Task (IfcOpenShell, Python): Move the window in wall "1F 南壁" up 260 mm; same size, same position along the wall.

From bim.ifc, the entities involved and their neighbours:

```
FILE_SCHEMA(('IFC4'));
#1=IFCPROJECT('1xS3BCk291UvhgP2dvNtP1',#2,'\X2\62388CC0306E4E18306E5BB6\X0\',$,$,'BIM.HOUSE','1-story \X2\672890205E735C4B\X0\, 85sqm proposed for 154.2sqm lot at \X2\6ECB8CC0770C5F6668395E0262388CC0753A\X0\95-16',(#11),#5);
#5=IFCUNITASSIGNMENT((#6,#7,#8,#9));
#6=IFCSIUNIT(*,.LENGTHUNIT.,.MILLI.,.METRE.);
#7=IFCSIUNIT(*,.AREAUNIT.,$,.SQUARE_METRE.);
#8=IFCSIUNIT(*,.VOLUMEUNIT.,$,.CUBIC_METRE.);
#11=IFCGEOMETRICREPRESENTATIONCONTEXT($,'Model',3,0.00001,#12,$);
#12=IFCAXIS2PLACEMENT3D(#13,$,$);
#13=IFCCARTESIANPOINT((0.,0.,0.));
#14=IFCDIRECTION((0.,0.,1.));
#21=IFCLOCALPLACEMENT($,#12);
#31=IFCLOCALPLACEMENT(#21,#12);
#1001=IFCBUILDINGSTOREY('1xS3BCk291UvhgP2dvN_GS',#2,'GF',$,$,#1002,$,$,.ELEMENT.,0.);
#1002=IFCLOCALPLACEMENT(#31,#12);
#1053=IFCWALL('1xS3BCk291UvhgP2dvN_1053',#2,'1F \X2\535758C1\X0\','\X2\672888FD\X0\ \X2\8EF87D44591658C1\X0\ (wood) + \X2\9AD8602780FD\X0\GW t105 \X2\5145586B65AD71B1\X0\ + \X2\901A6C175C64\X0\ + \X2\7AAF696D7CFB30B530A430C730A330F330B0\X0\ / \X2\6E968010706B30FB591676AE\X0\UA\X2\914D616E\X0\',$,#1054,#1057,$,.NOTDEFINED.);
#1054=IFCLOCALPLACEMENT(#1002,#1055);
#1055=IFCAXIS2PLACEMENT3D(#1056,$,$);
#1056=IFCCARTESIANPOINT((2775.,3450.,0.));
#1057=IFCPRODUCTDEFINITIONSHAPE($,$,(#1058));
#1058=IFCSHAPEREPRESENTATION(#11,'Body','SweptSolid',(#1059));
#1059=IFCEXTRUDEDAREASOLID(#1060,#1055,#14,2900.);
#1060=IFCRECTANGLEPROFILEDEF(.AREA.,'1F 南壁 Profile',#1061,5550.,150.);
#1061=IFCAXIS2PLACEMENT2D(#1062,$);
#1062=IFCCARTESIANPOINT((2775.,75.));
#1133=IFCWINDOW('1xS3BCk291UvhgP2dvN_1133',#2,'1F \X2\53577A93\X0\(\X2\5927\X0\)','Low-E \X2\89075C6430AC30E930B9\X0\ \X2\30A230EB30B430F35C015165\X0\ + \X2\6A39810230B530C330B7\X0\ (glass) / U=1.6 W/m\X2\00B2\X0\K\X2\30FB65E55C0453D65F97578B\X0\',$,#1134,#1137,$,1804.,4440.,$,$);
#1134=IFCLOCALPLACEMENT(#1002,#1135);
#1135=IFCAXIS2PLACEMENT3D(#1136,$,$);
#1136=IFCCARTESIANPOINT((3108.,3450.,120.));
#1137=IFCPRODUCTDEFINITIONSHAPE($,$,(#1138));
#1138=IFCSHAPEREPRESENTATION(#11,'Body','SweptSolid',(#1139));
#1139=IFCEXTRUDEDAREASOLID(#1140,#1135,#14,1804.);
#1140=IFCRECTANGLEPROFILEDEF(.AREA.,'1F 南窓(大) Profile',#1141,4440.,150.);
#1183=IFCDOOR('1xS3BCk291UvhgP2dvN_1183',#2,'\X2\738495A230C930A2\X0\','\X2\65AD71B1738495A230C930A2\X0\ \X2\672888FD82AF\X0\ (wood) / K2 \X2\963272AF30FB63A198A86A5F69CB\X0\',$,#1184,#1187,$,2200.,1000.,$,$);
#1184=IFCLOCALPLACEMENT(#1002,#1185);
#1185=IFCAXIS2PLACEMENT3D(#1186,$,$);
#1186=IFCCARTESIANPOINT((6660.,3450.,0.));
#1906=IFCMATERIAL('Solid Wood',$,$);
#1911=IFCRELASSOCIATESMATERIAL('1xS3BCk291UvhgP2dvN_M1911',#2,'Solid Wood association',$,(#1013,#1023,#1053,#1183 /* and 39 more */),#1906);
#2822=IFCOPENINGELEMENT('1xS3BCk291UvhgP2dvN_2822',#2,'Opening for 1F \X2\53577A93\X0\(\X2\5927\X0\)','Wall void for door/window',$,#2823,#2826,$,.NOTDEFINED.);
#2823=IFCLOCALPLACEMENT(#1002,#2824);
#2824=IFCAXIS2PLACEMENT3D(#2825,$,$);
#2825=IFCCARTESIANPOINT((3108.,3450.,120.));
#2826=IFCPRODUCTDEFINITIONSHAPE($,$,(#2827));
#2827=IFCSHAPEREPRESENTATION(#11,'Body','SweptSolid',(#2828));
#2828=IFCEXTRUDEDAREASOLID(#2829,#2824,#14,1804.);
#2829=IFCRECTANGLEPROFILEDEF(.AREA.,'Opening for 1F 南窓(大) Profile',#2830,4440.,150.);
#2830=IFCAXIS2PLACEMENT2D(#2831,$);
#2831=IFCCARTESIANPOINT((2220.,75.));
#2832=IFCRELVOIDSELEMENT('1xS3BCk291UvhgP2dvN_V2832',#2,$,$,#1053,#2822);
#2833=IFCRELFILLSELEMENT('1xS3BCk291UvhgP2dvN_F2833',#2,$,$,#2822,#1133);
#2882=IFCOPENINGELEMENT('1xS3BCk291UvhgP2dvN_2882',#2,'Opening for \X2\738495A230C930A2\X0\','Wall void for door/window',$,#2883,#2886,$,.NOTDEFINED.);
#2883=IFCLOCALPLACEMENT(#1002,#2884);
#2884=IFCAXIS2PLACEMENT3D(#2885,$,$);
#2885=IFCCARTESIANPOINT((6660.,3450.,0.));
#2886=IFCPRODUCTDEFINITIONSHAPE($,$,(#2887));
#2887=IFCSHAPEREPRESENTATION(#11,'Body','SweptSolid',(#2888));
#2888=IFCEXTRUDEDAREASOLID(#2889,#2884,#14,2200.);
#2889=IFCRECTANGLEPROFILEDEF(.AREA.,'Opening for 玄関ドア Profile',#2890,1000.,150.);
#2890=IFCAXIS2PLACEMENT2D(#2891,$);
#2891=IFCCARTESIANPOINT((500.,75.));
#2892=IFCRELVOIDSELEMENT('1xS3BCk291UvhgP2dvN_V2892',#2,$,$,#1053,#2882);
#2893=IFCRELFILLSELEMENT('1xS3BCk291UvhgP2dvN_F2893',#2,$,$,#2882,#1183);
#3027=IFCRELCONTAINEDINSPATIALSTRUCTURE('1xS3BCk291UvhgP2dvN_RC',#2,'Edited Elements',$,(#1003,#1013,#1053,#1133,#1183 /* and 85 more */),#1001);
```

```python
import numpy as np
import ifcopenshell
import ifcopenshell.api.geometry
import ifcopenshell.util.placement
import ifcopenshell.util.unit

model = ifcopenshell.open("bim.ifc")
unit_scale = ifcopenshell.util.unit.calculate_unit_scale(model)

window = model.by_guid("1xS3BCk291UvhgP2dvN_1133")
opening = window.FillsVoids[0].RelatingOpeningElement
dz = 0.26 / unit_scale

shift = np.array([0.0, 0.0, dz])
# The window is not placed relative to its opening, so move both.
for product in (opening, window):
    matrix = ifcopenshell.util.placement.get_local_placement(product.ObjectPlacement)
    matrix[:3, 3] += shift
    ifcopenshell.api.geometry.edit_object_placement(model, product=product, matrix=matrix, is_si=False)

print(f"moved by {dz * unit_scale:+.3f} m")

model.write("bim-out.ifc")
```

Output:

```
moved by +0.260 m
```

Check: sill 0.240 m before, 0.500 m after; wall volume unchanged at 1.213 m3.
